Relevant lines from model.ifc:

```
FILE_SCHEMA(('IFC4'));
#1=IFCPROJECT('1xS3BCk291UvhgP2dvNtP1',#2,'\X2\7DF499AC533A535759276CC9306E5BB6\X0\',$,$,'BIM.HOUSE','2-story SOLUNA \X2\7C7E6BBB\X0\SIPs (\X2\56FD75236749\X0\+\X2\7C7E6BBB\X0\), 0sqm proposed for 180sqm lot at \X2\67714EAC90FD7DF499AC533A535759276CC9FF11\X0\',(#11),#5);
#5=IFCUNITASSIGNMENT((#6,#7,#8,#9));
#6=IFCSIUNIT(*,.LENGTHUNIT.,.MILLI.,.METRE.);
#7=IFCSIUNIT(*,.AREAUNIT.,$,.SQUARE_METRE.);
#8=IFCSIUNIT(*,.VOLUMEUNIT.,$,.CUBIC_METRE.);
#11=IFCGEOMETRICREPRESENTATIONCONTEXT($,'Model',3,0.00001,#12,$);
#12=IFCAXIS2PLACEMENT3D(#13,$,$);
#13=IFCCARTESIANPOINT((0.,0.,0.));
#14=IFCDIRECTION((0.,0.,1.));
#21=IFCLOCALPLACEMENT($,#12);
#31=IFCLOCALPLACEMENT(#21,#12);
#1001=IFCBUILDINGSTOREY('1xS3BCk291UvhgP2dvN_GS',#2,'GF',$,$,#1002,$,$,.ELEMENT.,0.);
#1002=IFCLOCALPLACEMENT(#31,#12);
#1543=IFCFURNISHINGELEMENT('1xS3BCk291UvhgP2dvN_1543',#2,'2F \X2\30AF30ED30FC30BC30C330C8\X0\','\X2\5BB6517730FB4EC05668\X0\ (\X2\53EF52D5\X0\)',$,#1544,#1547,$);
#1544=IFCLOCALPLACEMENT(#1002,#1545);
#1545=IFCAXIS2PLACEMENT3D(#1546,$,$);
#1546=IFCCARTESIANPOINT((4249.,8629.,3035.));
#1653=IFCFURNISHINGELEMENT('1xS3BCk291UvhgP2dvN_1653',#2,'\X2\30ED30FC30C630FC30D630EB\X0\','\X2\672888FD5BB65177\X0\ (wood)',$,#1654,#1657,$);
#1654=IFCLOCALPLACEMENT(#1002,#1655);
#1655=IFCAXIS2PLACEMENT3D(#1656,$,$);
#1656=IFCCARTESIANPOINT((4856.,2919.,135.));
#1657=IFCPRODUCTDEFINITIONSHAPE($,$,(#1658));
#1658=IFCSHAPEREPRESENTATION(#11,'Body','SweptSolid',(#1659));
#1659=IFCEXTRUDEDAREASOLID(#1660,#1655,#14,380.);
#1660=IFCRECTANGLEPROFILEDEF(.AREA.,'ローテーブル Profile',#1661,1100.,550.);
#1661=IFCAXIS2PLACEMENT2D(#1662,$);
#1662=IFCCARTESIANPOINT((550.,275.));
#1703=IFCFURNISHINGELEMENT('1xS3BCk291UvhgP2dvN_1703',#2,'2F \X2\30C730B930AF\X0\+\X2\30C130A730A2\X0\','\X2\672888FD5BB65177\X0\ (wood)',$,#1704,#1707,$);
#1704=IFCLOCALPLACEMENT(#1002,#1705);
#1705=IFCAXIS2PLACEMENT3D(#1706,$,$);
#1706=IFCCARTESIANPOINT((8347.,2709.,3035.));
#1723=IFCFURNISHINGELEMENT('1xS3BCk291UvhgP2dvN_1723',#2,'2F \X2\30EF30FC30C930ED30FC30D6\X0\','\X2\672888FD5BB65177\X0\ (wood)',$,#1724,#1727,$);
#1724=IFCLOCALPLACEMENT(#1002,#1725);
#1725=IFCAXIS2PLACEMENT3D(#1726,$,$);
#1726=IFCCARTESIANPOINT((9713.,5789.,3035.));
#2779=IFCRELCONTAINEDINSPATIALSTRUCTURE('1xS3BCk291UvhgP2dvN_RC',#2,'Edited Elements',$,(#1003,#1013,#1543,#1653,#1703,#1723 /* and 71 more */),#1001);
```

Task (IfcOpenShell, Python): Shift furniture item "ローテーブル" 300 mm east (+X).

```python
import ifcopenshell
import ifcopenshell.api.geometry
import ifcopenshell.util.placement
import ifcopenshell.util.unit

model = ifcopenshell.open("model.ifc")
unit_scale = ifcopenshell.util.unit.calculate_unit_scale(model)

item = model.by_guid("1xS3BCk291UvhgP2dvN_1653")
matrix = ifcopenshell.util.placement.get_local_placement(item.ObjectPlacement)
matrix[0, 3] += 0.3 / unit_scale
ifcopenshell.api.geometry.edit_object_placement(model, product=item, matrix=matrix, is_si=False)

print(ifcopenshell.util.placement.get_local_placement(item.ObjectPlacement).round(3) + 0.0)

model.write("model_v2.ifc")
```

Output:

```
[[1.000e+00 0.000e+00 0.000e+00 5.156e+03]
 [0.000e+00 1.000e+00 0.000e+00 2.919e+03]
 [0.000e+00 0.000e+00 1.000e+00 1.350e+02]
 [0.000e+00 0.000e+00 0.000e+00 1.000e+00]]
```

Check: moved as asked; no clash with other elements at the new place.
